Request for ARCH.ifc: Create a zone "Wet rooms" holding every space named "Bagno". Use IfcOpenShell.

First a look at what the model holds.

```python
import ifcopenshell

model = ifcopenshell.open("ARCH.ifc")
print(model.schema)
seen = {}
for space in model.by_type("IfcSpace"):
    seen[space.LongName] = seen.get(space.LongName, 0) + 1
for name, count in sorted(seen.items(), key=str):
    print(count, "x", name)
print("zones:", [z.Name for z in model.by_type("IfcZone")][:20])
```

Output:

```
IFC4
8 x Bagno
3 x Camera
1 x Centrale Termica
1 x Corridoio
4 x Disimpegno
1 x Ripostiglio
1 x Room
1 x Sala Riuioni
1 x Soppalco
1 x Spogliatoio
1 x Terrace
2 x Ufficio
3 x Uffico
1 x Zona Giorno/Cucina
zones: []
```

```python
import ifcopenshell
import ifcopenshell.api.group
import ifcopenshell.api.root

model = ifcopenshell.open("ARCH.ifc")

names = {"Bagno"}
spaces = [s for s in model.by_type("IfcSpace") if s.LongName in names]

zone = ifcopenshell.api.root.create_entity(model, ifc_class="IfcZone", name="Wet rooms")
ifcopenshell.api.group.assign_group(model, products=spaces, group=zone)
print(len(spaces), "spaces in", zone.Name)

model.write("ARCH-out.ifc")
```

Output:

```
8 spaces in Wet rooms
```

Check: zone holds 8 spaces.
